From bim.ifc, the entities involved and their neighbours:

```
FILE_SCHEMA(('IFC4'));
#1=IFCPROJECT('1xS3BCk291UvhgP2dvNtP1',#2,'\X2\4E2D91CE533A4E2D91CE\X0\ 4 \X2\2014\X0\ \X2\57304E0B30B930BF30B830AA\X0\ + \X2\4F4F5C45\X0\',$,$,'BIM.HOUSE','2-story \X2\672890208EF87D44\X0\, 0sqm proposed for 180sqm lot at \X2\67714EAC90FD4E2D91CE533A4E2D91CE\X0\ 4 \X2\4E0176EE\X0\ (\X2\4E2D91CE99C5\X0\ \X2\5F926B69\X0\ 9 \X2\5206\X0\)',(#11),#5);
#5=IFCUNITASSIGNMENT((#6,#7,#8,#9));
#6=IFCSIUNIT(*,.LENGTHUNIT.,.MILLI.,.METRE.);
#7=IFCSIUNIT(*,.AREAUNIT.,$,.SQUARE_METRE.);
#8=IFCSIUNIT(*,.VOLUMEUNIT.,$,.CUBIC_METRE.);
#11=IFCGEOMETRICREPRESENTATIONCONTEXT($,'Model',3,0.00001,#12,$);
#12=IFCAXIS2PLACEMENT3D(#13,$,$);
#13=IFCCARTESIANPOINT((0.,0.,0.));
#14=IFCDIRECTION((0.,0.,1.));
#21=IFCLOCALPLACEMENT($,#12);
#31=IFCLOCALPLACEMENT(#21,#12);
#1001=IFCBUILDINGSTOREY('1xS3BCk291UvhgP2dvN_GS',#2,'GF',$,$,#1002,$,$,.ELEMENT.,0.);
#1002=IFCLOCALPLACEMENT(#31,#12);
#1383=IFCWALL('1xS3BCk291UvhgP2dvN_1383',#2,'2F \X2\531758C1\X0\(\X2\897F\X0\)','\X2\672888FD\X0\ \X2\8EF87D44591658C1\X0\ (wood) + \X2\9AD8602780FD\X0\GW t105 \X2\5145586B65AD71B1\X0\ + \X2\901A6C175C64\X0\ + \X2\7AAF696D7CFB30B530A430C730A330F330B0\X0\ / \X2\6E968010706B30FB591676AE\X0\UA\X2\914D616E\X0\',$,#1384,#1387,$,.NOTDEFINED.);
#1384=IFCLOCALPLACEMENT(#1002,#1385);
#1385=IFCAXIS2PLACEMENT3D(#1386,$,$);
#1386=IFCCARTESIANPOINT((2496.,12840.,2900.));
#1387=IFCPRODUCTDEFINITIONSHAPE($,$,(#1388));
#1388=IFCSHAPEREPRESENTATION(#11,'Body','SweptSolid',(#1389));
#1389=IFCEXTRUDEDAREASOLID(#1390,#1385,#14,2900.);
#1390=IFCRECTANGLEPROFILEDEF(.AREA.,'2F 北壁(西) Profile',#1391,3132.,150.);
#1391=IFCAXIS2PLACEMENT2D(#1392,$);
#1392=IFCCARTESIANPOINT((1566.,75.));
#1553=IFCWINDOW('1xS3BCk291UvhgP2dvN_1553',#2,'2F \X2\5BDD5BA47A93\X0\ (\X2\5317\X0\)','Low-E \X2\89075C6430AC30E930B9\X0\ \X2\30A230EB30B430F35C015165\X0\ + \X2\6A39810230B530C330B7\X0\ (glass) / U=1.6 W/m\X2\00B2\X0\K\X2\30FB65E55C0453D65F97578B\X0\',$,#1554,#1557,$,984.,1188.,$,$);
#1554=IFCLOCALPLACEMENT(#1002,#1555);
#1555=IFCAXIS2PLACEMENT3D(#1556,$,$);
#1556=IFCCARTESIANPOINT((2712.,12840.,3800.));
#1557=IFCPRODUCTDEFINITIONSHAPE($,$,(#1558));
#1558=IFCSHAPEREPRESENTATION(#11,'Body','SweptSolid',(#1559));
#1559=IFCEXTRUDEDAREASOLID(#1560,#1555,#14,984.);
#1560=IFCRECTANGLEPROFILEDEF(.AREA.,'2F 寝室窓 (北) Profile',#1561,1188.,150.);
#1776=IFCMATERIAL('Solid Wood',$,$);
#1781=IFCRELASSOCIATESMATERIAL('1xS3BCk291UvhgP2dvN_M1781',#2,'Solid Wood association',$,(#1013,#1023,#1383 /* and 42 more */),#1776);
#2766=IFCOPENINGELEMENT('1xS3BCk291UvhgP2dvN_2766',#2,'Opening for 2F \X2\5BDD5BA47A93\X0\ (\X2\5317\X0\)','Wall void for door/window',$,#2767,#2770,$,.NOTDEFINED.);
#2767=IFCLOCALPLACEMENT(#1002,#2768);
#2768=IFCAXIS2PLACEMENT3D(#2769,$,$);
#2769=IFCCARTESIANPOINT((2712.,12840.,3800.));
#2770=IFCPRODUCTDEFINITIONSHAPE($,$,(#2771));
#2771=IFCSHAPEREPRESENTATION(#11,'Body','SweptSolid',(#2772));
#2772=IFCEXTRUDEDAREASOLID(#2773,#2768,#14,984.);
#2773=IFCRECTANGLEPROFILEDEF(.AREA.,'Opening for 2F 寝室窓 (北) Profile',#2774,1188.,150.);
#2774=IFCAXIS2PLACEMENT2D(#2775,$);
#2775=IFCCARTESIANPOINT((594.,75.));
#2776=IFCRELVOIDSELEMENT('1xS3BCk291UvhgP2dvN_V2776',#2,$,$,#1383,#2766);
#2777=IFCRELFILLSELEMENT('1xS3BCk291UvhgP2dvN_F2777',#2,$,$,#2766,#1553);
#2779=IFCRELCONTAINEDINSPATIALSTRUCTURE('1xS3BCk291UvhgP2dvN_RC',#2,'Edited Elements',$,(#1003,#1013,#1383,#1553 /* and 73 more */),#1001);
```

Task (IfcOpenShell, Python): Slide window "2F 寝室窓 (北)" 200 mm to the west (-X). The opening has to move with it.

```python
import ifcopenshell
import ifcopenshell.api.geometry
import ifcopenshell.util.placement

model = ifcopenshell.open("bim.ifc")

window = model.by_id(1553)
opening = window.FillsVoids[0].RelatingOpeningElement
wall = opening.VoidsElements[0].RelatingBuildingElement

wall_matrix = ifcopenshell.util.placement.get_local_placement(wall.ObjectPlacement)
shift = wall_matrix[:3, 0] * -200.0
before = ifcopenshell.util.placement.get_local_placement(window.ObjectPlacement)[:3, 3].copy()

# The window is not placed relative to its opening, so move both.
for product in (opening, window):
    matrix = ifcopenshell.util.placement.get_local_placement(product.ObjectPlacement)
    matrix[:3, 3] += shift
    ifcopenshell.api.geometry.edit_object_placement(model, product=product, matrix=matrix, is_si=False)

after = ifcopenshell.util.placement.get_local_placement(window.ObjectPlacement)[:3, 3]
print("window moved by", (after - before).round(3) + 0.0)

model.write("bim-out.ifc")
```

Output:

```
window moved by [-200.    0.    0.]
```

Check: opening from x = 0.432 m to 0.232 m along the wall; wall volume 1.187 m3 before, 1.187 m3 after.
